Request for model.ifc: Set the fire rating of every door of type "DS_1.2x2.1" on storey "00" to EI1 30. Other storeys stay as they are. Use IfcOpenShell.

First a look at what the model holds.

```python
import ifcopenshell
import ifcopenshell.util.element

model = ifcopenshell.open("model.ifc")
print(model.schema)
storey = next(s for s in model.by_type("IfcBuildingStorey") if s.Name == "00")
doors = [e for e in ifcopenshell.util.element.get_decomposition(storey) if e.is_a("IfcDoor")]
seen = {}
for e in doors:
    element_type = ifcopenshell.util.element.get_type(e)
    key = (element_type.Name if element_type != e and element_type else None, ifcopenshell.util.element.get_pset(e, "Pset_DoorCommon", "FireRating"))
    seen[key] = seen.get(key, 0) + 1
for (name, value), count in sorted(seen.items(), key=str):
    print(count, "x", name, "|", value)
```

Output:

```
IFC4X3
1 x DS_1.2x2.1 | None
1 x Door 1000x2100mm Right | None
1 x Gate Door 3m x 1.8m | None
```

```python
import ifcopenshell
import ifcopenshell.api.pset
import ifcopenshell.util.element

model = ifcopenshell.open("model.ifc")

storey = next(s for s in model.by_type("IfcBuildingStorey") if s.Name == "00")
doors = [e for e in ifcopenshell.util.element.get_decomposition(storey) if e.is_a("IfcDoor")]

count = 0
for e in doors:
    element_type = ifcopenshell.util.element.get_type(e)
    if element_type in (None, e) or element_type.Name != "DS_1.2x2.1":
        continue
    # add_pset returns the element's existing set when there is one.
    pset = ifcopenshell.api.pset.add_pset(model, product=e, name="Pset_DoorCommon")
    ifcopenshell.api.pset.edit_pset(model, pset=pset, properties={"FireRating": "EI1 30"})
    count += 1

print(count, "doors updated")

model.write("model_rev.ifc")
```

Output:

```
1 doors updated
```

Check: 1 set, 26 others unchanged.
